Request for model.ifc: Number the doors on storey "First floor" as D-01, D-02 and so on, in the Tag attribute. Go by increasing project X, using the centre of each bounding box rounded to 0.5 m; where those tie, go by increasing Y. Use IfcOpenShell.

First a look at what the model holds.

```python
import ifcopenshell
import ifcopenshell.util.element
import ifcopenshell.util.placement

model = ifcopenshell.open("model.ifc")
print(model.schema)
storey = next(s for s in model.by_type("IfcBuildingStorey") if s.Name == "First floor")
doors = [e for e in ifcopenshell.util.element.get_decomposition(storey) if e.is_a("IfcDoor")]
for e in sorted(doors, key=lambda e: e.id()):
    origin = ifcopenshell.util.placement.get_local_placement(e.ObjectPlacement)[:3, 3]
    print(e.id(), e.Tag, e.Name, origin.round(2) + 0.0, sep=" | ")
```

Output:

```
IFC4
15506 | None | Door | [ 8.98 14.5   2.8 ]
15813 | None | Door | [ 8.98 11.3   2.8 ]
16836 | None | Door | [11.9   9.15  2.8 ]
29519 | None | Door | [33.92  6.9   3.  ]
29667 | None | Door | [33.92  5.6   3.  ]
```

```python
import ifcopenshell
import ifcopenshell.geom
import ifcopenshell.util.element
import ifcopenshell.util.shape

model = ifcopenshell.open("model.ifc")
settings = ifcopenshell.geom.settings()
settings.set("use-world-coords", True)


def centre(element):
    shape = ifcopenshell.geom.create_shape(settings, element)
    return ifcopenshell.util.shape.get_bbox_centroid(shape.geometry)


storey = next(s for s in model.by_type("IfcBuildingStorey") if s.Name == "First floor")
doors = [e for e in ifcopenshell.util.element.get_decomposition(storey) if e.is_a("IfcDoor")]

# Insertion points can sit at a corner or the storey origin, so sort by the geometry (in metres).
centres = {e: centre(e) for e in doors}
doors.sort(key=lambda e: (round(centres[e][0] / 0.5), centres[e][1]))

for i, e in enumerate(doors, start=1):
    number = f"D-{i:02d}"
    e.Tag = number
    print(e.id(), number)

model.write("model_updated.ifc")
```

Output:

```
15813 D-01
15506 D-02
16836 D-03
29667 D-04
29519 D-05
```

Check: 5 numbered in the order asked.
